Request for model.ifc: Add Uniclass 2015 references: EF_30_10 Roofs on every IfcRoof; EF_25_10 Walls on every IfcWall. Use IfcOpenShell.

First a look at what the model holds.

```python
import ifcopenshell

model = ifcopenshell.open("model.ifc")
print(model.schema)
print("classifications:", [c.Name for c in model.by_type("IfcClassification")])
for ifc_class in ("IfcDoor", "IfcRoof", "IfcStair", "IfcWall", "IfcWindow"):
    print(ifc_class, len(model.by_type(ifc_class)))
```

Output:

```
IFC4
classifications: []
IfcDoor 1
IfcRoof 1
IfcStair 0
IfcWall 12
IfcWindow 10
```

```python
import ifcopenshell
import ifcopenshell.api.classification

model = ifcopenshell.open("model.ifc")

system = ifcopenshell.api.classification.add_classification(model, classification="Uniclass 2015")

codes = {
    "IfcRoof": ("EF_30_10", "Roofs"),
    "IfcWall": ("EF_25_10", "Walls"),
}
for ifc_class, (code, name) in codes.items():
    products = model.by_type(ifc_class)
    ifcopenshell.api.classification.add_reference(
        model, products=products, classification=system, identification=code, name=name
    )
    print(code, len(products))

model.write("model_updated.ifc")
```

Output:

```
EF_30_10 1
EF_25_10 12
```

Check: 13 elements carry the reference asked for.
